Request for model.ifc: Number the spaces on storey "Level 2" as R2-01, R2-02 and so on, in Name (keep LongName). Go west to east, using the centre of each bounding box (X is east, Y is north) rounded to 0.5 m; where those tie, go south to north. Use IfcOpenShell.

First a look at what the model holds.

```python
import ifcopenshell
import ifcopenshell.util.element
import ifcopenshell.util.placement

model = ifcopenshell.open("model.ifc")
print(model.schema)
storey = next(s for s in model.by_type("IfcBuildingStorey") if s.Name == "Level 2")
spaces = [e for e in ifcopenshell.util.element.get_decomposition(storey) if e.is_a("IfcSpace")]
for e in sorted(spaces, key=lambda e: e.id()):
    origin = ifcopenshell.util.placement.get_local_placement(e.ObjectPlacement)[:3, 3]
    print(e.id(), e.Name, e.LongName, origin.round(2) + 0.0, sep=" | ")
```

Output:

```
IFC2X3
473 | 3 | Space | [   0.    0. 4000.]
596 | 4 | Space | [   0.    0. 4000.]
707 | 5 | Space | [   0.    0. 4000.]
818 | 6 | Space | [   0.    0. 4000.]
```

```python
import ifcopenshell
import ifcopenshell.geom
import ifcopenshell.util.element
import ifcopenshell.util.shape

model = ifcopenshell.open("model.ifc")
settings = ifcopenshell.geom.settings()
settings.set("use-world-coords", True)


def centre(element):
    shape = ifcopenshell.geom.create_shape(settings, element)
    return ifcopenshell.util.shape.get_bbox_centroid(shape.geometry)


storey = next(s for s in model.by_type("IfcBuildingStorey") if s.Name == "Level 2")
spaces = [e for e in ifcopenshell.util.element.get_decomposition(storey) if e.is_a("IfcSpace")]

# Insertion points can sit at a corner or the storey origin, so sort by the geometry (in metres).
centres = {e: centre(e) for e in spaces}
spaces.sort(key=lambda e: (round(centres[e][0] / 0.5), centres[e][1]))

for i, e in enumerate(spaces, start=1):
    number = f"R2-{i:02d}"
    e.Name = number
    print(e.id(), number)

model.write("model_updated.ifc")
```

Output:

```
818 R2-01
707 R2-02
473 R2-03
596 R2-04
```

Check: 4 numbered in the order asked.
